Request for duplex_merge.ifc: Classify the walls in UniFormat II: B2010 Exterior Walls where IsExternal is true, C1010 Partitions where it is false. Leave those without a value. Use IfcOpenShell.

First a look at what the model holds.

```python
import ifcopenshell
import ifcopenshell.util.element

model = ifcopenshell.open("duplex_merge.ifc")
print(model.schema)
print("classifications:", [c.Name for c in model.by_type("IfcClassification")])
values = [ifcopenshell.util.element.get_pset(e, "Pset_WallCommon", "IsExternal") for e in model.by_type("IfcWall")]
for value in (True, False, None):
    print("IsExternal", value, values.count(value))
```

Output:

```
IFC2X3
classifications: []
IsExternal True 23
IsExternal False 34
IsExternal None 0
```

```python
import ifcopenshell
import ifcopenshell.api.classification
import ifcopenshell.util.element

model = ifcopenshell.open("duplex_merge.ifc")

# IFC2X3 requires Source and Edition and has no link from the project to the system.
system = model.create_entity("IfcClassification", Source="ASTM", Edition="E1557", Name="UniFormat II")

walls = model.by_type("IfcWall")
external = {e: ifcopenshell.util.element.get_pset(e, "Pset_WallCommon", "IsExternal") for e in walls}
for flag, code, name in ((True, "B2010", "Exterior Walls"), (False, "C1010", "Partitions")):
    products = [e for e in walls if external[e] is flag]
    ifcopenshell.api.classification.add_reference(
        model, products=products, classification=system, identification=code, name=name
    )
    print(code, len(products))

model.write("duplex_merge_edited.ifc")
```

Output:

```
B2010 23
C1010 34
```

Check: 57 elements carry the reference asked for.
